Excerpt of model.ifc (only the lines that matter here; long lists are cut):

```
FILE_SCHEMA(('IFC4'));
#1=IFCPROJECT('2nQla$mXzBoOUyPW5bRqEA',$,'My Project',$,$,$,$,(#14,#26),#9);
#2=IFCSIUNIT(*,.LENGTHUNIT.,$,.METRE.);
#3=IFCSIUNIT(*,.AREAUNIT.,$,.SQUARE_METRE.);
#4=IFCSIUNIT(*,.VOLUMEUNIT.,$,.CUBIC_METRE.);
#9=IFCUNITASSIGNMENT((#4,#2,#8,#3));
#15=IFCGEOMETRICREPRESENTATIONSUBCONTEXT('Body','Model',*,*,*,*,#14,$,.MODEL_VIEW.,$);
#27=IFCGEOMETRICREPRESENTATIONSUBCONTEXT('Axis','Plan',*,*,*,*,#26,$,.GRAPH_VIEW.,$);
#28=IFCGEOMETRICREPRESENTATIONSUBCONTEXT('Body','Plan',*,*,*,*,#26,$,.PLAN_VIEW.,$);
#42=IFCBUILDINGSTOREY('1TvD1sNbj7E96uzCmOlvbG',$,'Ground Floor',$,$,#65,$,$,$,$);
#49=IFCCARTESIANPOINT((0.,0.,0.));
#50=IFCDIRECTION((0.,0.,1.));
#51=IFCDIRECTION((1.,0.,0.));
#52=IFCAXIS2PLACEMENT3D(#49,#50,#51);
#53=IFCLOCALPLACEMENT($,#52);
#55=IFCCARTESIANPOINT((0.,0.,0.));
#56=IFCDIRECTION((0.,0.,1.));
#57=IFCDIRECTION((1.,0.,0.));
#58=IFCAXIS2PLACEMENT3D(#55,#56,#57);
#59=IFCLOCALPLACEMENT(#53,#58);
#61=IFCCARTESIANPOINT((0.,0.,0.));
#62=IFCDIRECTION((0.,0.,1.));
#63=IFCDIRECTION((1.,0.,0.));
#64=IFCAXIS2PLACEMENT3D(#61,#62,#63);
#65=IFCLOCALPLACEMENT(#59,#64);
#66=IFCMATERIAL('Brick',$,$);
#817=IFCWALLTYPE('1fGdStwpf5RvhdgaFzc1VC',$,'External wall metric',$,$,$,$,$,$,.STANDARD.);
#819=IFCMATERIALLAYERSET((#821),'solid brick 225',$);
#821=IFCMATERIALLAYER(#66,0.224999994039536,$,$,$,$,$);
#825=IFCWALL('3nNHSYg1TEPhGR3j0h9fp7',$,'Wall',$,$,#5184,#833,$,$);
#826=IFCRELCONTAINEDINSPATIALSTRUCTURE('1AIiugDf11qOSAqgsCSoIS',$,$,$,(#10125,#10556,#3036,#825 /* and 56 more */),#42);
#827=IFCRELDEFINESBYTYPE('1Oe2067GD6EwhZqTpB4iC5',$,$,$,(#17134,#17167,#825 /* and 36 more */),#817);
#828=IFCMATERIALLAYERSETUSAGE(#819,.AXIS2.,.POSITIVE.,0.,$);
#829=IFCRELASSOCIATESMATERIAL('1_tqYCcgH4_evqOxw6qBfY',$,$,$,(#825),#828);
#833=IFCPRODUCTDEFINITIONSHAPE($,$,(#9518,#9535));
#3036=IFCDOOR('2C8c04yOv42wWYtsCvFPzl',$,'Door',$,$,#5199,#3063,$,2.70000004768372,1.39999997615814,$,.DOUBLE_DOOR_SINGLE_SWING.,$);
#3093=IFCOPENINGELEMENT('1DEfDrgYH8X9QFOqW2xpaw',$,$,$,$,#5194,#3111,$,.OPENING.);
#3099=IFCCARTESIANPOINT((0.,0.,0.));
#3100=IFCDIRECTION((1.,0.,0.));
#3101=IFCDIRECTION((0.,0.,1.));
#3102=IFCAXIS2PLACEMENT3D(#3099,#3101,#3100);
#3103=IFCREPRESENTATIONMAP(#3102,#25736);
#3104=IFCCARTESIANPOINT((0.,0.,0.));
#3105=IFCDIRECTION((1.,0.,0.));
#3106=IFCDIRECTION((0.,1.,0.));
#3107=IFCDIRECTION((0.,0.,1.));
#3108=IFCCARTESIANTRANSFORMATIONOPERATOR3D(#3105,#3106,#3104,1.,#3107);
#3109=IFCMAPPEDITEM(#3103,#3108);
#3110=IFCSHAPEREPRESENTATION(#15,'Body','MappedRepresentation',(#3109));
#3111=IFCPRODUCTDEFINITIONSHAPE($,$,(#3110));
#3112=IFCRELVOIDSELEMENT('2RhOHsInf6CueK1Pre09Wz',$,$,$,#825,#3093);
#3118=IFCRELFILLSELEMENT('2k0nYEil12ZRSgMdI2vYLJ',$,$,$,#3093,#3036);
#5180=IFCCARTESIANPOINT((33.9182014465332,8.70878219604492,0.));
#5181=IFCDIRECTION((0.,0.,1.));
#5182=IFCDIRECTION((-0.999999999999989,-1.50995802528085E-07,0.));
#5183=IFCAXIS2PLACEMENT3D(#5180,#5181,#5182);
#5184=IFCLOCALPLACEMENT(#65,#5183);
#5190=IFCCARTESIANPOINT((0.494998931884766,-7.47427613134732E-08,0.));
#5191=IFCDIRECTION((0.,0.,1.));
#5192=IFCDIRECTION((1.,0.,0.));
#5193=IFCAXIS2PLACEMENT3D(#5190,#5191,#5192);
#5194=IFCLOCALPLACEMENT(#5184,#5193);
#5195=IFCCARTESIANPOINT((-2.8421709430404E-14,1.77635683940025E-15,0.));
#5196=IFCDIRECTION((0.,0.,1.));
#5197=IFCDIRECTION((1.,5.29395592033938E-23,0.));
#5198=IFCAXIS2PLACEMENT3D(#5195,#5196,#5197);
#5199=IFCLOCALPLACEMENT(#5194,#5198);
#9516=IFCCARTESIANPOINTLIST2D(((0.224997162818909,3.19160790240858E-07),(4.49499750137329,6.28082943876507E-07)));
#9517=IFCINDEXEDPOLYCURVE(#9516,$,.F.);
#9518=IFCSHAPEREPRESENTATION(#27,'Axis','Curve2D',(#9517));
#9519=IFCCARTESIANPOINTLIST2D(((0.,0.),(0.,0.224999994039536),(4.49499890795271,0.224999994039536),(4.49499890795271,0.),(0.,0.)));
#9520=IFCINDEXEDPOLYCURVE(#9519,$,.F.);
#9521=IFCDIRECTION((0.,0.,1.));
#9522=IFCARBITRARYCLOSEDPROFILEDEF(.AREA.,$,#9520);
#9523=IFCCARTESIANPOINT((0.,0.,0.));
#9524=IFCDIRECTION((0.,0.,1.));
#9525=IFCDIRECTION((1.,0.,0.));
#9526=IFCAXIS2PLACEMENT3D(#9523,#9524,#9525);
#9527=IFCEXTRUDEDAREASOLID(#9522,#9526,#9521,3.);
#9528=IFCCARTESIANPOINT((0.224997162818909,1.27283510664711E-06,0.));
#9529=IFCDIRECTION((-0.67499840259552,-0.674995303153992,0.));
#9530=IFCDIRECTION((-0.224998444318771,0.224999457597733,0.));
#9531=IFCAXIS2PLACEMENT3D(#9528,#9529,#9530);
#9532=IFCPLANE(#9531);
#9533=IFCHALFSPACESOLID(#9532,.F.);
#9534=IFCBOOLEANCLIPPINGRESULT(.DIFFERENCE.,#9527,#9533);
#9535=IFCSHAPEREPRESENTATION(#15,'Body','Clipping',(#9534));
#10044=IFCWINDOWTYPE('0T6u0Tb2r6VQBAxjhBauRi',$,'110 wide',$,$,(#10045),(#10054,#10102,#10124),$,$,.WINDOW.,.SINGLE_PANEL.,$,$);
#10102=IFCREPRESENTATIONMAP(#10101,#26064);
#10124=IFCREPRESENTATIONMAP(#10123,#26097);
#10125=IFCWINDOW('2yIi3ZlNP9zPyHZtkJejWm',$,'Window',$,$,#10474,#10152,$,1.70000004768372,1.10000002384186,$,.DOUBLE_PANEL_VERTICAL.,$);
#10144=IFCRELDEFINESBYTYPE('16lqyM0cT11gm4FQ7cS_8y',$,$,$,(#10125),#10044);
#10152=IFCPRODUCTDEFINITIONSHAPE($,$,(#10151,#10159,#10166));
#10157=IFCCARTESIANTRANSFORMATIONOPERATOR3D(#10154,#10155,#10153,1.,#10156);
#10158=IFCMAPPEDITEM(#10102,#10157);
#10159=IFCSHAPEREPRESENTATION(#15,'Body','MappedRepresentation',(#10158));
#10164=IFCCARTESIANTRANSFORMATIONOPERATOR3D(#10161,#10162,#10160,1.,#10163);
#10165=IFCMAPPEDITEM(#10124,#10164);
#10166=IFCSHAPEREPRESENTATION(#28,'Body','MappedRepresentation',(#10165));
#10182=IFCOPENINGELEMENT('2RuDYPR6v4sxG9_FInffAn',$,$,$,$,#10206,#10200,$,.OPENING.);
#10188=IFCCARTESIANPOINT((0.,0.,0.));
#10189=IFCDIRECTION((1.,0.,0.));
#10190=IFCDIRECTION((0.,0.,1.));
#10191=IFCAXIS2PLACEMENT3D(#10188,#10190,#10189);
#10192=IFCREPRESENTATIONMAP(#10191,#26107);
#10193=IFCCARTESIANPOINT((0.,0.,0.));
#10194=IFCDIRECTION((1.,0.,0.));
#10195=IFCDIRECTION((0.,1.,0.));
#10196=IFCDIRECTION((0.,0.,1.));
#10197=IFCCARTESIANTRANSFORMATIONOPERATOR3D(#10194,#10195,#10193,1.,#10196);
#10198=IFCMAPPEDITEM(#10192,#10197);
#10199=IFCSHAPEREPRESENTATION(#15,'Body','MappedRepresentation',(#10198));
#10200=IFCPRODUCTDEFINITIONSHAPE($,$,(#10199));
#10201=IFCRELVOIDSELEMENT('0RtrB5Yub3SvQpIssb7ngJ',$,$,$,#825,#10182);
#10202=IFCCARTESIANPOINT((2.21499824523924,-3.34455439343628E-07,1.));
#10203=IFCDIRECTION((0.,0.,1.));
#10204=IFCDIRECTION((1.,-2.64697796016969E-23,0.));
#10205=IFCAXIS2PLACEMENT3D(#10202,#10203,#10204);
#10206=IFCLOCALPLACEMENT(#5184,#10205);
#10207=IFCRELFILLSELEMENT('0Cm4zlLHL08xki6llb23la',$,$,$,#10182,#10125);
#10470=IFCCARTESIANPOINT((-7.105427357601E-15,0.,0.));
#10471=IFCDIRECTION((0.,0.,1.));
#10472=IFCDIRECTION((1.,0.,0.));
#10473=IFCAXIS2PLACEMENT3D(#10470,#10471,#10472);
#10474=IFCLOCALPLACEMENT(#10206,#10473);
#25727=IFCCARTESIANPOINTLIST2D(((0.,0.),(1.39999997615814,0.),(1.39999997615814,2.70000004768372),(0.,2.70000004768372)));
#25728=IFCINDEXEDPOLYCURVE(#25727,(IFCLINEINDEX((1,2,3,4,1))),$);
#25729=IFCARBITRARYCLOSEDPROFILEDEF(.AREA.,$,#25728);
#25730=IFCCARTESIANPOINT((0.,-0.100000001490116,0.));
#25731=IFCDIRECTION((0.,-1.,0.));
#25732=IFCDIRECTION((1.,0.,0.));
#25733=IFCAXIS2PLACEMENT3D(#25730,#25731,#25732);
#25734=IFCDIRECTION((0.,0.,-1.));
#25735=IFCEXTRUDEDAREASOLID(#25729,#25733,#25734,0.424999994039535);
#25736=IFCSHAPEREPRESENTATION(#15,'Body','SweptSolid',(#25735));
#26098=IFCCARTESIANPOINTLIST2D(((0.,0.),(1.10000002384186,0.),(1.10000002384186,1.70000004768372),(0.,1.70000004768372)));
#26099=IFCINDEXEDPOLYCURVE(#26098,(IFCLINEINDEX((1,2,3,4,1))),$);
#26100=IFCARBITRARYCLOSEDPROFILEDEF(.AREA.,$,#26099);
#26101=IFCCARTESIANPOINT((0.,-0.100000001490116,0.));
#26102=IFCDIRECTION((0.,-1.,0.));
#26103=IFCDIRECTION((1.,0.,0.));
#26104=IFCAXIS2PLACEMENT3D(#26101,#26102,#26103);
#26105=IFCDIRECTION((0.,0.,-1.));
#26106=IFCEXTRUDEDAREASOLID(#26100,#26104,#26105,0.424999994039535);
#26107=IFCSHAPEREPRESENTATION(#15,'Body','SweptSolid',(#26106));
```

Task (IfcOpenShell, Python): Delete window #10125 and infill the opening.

```python
import ifcopenshell
import ifcopenshell.api.feature
import ifcopenshell.api.root
import ifcopenshell.geom
import ifcopenshell.util.shape

model = ifcopenshell.open("model.ifc")
settings = ifcopenshell.geom.settings()


def volume(element):
    """Net volume in cubic metres, openings subtracted."""
    shape = ifcopenshell.geom.create_shape(settings, element)
    return ifcopenshell.util.shape.get_volume(shape.geometry)


window = model.by_guid("2yIi3ZlNP9zPyHZtkJejWm")
opening = window.FillsVoids[0].RelatingOpeningElement
wall = opening.VoidsElements[0].RelatingBuildingElement
before = volume(wall)

ifcopenshell.api.root.remove_product(model, product=window)
ifcopenshell.api.feature.remove_feature(model, feature=opening)

after = volume(wall)

print(f"wall volume {before:.3f} -> {after:.3f} m3")

model.write("model-out.ifc")
```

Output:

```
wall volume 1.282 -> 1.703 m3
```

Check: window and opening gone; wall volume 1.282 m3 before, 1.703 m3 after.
